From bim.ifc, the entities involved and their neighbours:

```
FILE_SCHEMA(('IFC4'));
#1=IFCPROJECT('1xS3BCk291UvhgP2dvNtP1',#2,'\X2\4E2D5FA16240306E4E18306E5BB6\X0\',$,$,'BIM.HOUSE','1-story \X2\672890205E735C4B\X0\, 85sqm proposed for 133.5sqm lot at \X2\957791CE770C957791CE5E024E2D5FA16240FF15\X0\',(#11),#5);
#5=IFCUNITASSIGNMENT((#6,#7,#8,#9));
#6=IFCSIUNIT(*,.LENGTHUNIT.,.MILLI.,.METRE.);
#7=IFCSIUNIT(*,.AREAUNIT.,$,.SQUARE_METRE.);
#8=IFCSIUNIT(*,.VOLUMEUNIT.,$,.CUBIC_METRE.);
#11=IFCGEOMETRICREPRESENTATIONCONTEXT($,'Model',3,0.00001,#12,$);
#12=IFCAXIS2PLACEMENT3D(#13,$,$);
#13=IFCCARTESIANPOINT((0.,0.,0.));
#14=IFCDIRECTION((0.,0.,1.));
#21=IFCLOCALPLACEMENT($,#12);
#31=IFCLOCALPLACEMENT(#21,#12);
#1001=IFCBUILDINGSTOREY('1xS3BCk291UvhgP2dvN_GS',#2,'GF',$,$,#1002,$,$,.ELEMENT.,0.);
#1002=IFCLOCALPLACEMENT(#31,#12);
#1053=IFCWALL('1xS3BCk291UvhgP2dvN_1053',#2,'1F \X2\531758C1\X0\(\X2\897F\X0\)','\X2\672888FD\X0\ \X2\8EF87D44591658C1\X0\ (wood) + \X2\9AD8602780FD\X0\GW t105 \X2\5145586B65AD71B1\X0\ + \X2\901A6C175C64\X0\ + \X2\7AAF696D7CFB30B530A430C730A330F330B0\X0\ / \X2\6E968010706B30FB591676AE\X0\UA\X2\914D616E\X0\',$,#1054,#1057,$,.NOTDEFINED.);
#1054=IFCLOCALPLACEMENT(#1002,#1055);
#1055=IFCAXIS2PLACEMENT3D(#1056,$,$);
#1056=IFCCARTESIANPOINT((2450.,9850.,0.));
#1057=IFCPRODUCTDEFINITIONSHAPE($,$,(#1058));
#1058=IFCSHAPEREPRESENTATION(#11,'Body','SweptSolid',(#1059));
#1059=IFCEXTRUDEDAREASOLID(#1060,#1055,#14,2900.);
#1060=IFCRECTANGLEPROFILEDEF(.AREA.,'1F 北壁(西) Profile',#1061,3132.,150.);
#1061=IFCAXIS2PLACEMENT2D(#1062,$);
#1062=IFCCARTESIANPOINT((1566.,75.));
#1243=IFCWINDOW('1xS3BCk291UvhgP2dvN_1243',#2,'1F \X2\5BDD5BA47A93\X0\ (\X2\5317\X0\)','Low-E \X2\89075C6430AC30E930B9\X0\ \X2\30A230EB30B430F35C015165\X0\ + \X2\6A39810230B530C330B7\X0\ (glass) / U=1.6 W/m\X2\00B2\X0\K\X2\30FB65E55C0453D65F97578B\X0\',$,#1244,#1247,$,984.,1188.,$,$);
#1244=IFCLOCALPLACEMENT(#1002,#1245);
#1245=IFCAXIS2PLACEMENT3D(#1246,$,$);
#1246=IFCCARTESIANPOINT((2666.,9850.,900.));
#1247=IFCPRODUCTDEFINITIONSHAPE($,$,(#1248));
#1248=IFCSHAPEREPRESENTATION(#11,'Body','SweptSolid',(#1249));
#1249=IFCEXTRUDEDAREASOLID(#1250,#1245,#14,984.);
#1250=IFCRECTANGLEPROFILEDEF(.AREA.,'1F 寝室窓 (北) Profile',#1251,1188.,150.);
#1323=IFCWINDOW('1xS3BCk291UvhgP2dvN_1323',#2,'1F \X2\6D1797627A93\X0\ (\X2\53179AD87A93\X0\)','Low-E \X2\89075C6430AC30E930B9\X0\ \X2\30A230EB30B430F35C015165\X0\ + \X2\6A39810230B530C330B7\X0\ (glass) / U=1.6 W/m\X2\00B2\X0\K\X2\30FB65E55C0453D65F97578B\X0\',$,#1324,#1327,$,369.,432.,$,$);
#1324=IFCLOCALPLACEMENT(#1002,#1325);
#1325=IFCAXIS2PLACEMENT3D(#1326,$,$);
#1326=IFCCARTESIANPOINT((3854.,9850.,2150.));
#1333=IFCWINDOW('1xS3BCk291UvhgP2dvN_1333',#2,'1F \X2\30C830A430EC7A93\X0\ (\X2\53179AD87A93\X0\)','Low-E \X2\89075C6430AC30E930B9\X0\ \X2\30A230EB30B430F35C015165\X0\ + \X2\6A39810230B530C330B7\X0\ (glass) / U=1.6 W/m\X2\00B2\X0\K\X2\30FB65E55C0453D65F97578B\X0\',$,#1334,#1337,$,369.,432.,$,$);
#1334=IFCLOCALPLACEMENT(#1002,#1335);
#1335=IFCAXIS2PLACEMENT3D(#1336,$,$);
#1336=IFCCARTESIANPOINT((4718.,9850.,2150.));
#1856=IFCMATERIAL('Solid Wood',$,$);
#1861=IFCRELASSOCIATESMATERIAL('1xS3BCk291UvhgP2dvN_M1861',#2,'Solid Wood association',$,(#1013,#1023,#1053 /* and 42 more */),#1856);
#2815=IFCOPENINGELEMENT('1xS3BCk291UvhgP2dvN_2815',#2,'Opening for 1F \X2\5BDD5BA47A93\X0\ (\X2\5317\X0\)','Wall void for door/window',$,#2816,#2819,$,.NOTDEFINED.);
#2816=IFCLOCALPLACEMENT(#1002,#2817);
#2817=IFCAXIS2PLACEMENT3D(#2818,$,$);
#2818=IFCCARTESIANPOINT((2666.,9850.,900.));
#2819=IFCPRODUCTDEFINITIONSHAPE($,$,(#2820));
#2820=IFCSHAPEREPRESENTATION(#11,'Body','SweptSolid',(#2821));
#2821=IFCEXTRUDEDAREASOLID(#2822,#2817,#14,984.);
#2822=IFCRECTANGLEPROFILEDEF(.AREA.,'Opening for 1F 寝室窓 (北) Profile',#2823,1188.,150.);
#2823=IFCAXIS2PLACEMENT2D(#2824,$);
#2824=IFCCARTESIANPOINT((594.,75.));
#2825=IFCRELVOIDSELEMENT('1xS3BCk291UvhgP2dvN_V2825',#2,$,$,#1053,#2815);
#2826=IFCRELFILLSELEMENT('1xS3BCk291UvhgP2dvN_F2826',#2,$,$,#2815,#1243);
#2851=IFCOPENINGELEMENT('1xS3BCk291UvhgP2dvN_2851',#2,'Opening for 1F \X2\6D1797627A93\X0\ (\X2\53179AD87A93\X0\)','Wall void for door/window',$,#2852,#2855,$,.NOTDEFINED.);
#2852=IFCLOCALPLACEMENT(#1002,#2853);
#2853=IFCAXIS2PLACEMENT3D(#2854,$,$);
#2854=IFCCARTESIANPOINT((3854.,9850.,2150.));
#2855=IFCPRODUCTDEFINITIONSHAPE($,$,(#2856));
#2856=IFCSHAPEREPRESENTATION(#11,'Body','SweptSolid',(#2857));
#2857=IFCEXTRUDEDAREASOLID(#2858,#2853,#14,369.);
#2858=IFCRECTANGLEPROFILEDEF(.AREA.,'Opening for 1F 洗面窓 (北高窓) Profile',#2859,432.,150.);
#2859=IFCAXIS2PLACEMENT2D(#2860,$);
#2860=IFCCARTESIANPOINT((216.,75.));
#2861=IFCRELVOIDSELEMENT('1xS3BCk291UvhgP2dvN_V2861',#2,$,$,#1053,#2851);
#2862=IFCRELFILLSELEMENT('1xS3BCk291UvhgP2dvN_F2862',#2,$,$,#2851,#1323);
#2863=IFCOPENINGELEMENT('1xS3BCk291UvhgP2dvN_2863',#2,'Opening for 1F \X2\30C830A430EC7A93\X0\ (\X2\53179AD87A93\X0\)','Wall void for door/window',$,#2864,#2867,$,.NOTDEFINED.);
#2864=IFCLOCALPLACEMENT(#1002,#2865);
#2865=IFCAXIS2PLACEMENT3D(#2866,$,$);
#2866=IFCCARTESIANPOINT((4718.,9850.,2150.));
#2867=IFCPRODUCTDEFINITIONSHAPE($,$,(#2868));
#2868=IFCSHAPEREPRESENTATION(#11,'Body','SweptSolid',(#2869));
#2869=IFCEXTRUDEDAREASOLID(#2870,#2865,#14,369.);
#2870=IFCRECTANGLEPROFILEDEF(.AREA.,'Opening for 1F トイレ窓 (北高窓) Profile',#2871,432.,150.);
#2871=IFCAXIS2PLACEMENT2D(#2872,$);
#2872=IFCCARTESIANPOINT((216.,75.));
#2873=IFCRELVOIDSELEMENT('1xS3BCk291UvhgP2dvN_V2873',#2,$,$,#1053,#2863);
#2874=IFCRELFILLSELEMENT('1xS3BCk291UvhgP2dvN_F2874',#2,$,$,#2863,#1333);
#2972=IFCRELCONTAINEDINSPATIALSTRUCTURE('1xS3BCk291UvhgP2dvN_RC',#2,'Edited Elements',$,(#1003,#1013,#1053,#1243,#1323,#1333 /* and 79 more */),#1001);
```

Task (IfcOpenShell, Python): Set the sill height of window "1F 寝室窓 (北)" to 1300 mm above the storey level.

```python
import numpy as np
import ifcopenshell
import ifcopenshell.api.geometry
import ifcopenshell.geom
import ifcopenshell.util.element
import ifcopenshell.util.placement
import ifcopenshell.util.shape
import ifcopenshell.util.unit

model = ifcopenshell.open("bim.ifc")
unit_scale = ifcopenshell.util.unit.calculate_unit_scale(model)

window = model.by_id(1243)
opening = window.FillsVoids[0].RelatingOpeningElement
storey = ifcopenshell.util.element.get_container(window, ifc_class="IfcBuildingStorey")
level = ifcopenshell.util.placement.get_local_placement(storey.ObjectPlacement)[2, 3]

# The opening's origin need not be at the sill, so measure its lowest point.
shape = ifcopenshell.geom.create_shape(ifcopenshell.geom.settings(), opening)
bottom = ifcopenshell.util.shape.get_shape_bottom_elevation(shape, shape.geometry) / unit_scale
dz = level + 1300.0 - bottom

shift = np.array([0.0, 0.0, dz])
# The window is not placed relative to its opening, so move both.
for product in (opening, window):
    matrix = ifcopenshell.util.placement.get_local_placement(product.ObjectPlacement)
    matrix[:3, 3] += shift
    ifcopenshell.api.geometry.edit_object_placement(model, product=product, matrix=matrix, is_si=False)

print(f"moved by {dz * unit_scale:+.3f} m")

model.write("bim_edited.ifc")
```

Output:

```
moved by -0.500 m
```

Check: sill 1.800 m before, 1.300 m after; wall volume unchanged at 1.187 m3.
